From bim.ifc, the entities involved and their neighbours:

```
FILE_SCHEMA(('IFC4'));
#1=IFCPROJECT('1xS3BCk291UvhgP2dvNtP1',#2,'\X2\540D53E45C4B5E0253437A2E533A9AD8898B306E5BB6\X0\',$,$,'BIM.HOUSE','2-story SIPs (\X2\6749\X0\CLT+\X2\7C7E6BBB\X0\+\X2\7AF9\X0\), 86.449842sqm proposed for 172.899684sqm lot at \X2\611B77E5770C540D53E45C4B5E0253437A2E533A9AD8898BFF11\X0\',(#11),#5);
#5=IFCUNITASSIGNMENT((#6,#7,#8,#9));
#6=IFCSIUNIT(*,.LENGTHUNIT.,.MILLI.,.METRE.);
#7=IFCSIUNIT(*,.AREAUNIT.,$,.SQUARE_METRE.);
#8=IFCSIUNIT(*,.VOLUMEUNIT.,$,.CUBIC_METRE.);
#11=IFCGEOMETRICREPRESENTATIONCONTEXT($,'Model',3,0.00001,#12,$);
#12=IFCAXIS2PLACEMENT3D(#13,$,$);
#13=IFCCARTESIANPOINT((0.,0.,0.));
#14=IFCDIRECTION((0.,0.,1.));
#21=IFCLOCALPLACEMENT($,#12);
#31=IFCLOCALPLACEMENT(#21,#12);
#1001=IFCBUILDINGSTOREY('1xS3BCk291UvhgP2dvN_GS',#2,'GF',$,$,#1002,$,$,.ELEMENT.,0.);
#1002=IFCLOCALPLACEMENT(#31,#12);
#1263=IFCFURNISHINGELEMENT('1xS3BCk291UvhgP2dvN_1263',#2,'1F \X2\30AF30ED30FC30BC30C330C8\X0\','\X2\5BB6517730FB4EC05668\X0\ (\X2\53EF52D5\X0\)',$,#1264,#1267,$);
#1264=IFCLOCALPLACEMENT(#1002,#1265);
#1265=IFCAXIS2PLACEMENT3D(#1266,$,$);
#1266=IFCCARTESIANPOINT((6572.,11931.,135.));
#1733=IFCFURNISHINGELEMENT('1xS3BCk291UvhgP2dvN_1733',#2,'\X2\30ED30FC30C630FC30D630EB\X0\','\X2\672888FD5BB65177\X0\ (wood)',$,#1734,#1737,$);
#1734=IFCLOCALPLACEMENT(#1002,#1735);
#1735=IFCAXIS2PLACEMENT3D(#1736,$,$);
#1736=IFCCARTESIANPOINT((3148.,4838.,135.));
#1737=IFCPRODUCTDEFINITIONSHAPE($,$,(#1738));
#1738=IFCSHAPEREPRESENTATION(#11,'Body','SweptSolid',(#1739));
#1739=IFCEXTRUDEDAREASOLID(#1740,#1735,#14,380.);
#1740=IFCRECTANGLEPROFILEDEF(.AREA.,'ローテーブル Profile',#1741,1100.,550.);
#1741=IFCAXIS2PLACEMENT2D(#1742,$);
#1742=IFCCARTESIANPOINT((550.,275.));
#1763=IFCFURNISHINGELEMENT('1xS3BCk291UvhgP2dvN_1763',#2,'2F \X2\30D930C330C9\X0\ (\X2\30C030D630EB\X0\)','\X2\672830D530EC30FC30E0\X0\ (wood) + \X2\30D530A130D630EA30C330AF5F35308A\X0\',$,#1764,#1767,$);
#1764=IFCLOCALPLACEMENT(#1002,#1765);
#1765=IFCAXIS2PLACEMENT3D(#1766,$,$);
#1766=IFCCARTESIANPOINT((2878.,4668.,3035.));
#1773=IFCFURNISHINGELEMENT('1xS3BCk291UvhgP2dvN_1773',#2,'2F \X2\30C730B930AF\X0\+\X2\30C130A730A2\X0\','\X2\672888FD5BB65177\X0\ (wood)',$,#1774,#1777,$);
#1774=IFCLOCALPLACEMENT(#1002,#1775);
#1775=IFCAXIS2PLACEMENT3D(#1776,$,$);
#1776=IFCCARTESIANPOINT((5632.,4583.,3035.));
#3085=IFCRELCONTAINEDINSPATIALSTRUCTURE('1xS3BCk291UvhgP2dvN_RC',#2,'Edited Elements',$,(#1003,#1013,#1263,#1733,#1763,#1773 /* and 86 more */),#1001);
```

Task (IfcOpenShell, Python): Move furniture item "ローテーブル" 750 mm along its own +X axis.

```python
import ifcopenshell
import ifcopenshell.api.geometry
import ifcopenshell.util.placement

model = ifcopenshell.open("bim.ifc")

item = model.by_guid("1xS3BCk291UvhgP2dvN_1733")
matrix = ifcopenshell.util.placement.get_local_placement(item.ObjectPlacement)
matrix[:3, 3] += matrix[:3, 0] * 750.0
ifcopenshell.api.geometry.edit_object_placement(model, product=item, matrix=matrix, is_si=False)

print(ifcopenshell.util.placement.get_local_placement(item.ObjectPlacement).round(3) + 0.0)

model.write("bim_edited.ifc")
```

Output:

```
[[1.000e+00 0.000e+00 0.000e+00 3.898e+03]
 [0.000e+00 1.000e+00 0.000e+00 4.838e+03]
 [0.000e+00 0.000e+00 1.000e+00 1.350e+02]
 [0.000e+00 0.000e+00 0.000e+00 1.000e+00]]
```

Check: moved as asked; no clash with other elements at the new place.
